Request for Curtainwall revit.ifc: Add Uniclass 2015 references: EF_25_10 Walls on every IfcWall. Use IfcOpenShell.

First a look at what the model holds.

```python
import ifcopenshell

model = ifcopenshell.open("Curtainwall revit.ifc")
print(model.schema)
print("classifications:", [c.Name for c in model.by_type("IfcClassification")])
for ifc_class in ("IfcDoor", "IfcRoof", "IfcStair", "IfcWall", "IfcWindow"):
    print(ifc_class, len(model.by_type(ifc_class)))
```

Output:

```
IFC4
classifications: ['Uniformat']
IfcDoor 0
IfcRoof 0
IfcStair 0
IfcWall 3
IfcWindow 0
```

```python
import ifcopenshell
import ifcopenshell.api.classification

model = ifcopenshell.open("Curtainwall revit.ifc")

system = ifcopenshell.api.classification.add_classification(model, classification="Uniclass 2015")

codes = {
    "IfcWall": ("EF_25_10", "Walls"),
}
for ifc_class, (code, name) in codes.items():
    products = model.by_type(ifc_class)
    ifcopenshell.api.classification.add_reference(
        model, products=products, classification=system, identification=code, name=name
    )
    print(code, len(products))

model.write("Curtainwall revit_updated.ifc")
```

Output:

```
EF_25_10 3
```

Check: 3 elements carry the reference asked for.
